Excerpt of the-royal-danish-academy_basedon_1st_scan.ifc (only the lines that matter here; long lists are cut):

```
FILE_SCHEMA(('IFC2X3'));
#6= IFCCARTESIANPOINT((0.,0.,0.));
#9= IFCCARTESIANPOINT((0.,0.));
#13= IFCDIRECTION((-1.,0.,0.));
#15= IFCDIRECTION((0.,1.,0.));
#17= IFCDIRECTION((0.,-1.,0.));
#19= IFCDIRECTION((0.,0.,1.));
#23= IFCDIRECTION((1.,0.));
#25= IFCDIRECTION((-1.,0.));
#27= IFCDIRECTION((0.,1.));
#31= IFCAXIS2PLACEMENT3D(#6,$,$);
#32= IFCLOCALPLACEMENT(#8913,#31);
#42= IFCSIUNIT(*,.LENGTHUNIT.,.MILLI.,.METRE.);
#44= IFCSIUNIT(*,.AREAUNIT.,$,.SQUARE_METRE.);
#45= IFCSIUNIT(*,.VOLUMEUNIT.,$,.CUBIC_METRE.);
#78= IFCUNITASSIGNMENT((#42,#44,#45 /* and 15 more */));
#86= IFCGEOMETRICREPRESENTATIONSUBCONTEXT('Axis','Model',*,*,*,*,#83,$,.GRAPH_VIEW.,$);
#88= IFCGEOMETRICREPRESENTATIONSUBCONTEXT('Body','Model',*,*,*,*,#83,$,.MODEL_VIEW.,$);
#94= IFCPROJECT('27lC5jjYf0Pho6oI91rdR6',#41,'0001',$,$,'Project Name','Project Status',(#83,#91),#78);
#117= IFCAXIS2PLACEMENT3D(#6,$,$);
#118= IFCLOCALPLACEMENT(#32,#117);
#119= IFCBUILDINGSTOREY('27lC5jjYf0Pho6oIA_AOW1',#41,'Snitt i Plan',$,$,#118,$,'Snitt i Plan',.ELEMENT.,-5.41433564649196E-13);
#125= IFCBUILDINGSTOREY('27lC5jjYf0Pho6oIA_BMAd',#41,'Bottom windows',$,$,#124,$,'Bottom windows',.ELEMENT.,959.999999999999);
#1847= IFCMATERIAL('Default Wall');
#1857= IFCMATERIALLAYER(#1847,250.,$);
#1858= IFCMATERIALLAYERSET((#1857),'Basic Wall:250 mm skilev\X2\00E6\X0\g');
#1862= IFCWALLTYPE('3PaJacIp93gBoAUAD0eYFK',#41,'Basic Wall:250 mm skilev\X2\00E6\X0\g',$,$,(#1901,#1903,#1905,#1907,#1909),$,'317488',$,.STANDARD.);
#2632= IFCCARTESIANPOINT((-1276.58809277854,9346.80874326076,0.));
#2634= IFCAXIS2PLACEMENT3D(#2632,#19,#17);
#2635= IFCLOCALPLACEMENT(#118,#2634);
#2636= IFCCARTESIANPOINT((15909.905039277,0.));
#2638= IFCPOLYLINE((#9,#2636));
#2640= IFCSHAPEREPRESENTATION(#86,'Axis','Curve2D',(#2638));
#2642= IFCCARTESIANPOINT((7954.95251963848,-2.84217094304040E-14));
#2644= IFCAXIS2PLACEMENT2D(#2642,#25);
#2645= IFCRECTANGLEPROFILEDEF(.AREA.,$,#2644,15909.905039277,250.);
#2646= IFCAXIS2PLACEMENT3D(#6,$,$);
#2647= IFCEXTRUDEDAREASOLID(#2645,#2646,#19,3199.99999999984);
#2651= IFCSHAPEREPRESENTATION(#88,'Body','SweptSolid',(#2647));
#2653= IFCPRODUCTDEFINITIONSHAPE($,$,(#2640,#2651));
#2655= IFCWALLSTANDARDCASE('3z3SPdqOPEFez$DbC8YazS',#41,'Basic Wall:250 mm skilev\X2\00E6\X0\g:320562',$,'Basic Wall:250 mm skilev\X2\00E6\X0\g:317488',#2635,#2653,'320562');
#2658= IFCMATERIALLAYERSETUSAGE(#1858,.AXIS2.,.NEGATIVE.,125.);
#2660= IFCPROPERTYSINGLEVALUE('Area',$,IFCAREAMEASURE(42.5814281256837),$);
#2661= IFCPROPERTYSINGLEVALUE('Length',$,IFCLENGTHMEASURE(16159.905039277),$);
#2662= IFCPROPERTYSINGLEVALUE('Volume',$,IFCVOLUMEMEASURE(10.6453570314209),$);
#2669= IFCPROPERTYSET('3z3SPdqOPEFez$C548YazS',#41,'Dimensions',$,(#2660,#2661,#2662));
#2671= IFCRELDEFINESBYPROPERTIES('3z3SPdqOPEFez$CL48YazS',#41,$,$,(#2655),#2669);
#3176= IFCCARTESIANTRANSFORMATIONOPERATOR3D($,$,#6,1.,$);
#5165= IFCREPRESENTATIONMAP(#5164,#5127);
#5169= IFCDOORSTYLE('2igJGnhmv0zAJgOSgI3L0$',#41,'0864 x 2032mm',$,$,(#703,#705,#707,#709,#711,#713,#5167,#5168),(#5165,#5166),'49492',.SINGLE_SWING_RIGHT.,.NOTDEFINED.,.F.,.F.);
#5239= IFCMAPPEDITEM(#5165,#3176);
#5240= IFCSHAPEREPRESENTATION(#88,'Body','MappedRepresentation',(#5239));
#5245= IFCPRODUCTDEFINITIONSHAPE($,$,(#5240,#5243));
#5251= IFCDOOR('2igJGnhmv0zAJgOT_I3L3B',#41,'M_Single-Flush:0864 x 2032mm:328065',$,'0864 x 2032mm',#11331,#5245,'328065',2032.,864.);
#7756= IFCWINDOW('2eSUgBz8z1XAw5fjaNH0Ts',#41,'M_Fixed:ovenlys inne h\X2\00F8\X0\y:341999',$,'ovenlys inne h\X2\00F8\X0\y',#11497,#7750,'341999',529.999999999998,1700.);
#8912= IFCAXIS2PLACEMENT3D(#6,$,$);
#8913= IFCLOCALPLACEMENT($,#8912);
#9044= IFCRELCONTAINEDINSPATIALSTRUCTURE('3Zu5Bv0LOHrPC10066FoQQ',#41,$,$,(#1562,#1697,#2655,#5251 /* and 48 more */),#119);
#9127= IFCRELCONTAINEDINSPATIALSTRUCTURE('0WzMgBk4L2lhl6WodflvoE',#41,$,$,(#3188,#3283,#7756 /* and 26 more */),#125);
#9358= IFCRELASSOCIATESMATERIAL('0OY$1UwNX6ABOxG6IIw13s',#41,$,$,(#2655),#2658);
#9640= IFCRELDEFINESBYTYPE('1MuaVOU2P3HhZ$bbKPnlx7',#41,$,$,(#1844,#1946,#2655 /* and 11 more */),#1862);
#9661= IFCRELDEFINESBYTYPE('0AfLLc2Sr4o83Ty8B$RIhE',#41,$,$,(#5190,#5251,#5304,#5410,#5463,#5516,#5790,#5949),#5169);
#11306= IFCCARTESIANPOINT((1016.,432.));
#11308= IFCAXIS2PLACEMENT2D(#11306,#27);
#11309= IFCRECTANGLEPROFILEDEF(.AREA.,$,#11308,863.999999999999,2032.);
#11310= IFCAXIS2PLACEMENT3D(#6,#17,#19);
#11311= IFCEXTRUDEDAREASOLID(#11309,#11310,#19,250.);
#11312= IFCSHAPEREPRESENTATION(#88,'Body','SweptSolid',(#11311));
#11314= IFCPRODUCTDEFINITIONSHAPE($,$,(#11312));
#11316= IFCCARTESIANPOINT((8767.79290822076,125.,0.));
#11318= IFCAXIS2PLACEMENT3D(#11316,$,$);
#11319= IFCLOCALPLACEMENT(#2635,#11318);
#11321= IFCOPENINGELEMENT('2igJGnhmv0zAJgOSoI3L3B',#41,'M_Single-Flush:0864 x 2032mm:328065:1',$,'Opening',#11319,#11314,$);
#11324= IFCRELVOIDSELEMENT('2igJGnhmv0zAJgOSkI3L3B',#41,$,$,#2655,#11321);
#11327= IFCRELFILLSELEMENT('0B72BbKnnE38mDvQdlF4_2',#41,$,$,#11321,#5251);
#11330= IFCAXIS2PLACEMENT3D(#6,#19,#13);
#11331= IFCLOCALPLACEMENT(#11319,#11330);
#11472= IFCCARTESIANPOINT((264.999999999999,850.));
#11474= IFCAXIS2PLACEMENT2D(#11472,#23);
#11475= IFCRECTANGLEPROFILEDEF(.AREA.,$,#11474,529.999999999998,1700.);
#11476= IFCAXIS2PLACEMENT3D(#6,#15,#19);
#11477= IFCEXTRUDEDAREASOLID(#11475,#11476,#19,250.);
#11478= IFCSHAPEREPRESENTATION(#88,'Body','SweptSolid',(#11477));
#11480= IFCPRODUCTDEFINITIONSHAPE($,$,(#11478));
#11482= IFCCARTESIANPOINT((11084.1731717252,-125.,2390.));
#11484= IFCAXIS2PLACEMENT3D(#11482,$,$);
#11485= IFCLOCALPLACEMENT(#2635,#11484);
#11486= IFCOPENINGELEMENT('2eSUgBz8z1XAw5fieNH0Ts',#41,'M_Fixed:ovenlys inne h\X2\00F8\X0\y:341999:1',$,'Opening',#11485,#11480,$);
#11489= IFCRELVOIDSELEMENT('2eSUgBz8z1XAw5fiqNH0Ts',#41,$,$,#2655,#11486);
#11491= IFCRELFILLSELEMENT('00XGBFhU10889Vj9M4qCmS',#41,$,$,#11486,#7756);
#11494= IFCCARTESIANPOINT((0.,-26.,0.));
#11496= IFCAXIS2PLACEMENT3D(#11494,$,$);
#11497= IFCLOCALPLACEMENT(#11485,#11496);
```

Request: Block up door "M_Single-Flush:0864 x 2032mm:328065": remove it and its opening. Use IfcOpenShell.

```python
import ifcopenshell
import ifcopenshell.api.feature
import ifcopenshell.api.pset
import ifcopenshell.api.root
import ifcopenshell.geom
import ifcopenshell.util.element
import ifcopenshell.util.shape
import ifcopenshell.util.unit

model = ifcopenshell.open("the-royal-danish-academy_basedon_1st_scan.ifc")
area_scale = ifcopenshell.util.unit.calculate_unit_scale(model, "AREAUNIT")
volume_scale = ifcopenshell.util.unit.calculate_unit_scale(model, "VOLUMEUNIT")
settings = ifcopenshell.geom.settings()


def volume(element):
    """Net volume in cubic metres, openings subtracted."""
    shape = ifcopenshell.geom.create_shape(settings, element)
    return ifcopenshell.util.shape.get_volume(shape.geometry)


door = model.by_guid("2igJGnhmv0zAJgOT_I3L3B")
opening = door.FillsVoids[0].RelatingOpeningElement
wall = opening.VoidsElements[0].RelatingBuildingElement
before = volume(wall)

ifcopenshell.api.root.remove_product(model, product=door)
ifcopenshell.api.feature.remove_feature(model, feature=opening)

after = volume(wall)
thickness = 0.25  # wall thickness in metres

# Update the wall's stored quantities.
pset = model.by_id(ifcopenshell.util.element.get_pset(wall, "Dimensions", should_inherit=False)["id"])
ifcopenshell.api.pset.edit_pset(model, pset=pset, properties={
    "Area": model.create_entity("IfcAreaMeasure", after / thickness / area_scale),
    "Volume": model.create_entity("IfcVolumeMeasure", after / volume_scale),
})

print(f"wall volume {before:.3f} -> {after:.3f} m3")

model.write("the-royal-danish-academy_basedon_1st_scan_rev.ifc")
```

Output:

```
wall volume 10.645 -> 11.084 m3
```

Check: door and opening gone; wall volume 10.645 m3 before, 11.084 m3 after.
